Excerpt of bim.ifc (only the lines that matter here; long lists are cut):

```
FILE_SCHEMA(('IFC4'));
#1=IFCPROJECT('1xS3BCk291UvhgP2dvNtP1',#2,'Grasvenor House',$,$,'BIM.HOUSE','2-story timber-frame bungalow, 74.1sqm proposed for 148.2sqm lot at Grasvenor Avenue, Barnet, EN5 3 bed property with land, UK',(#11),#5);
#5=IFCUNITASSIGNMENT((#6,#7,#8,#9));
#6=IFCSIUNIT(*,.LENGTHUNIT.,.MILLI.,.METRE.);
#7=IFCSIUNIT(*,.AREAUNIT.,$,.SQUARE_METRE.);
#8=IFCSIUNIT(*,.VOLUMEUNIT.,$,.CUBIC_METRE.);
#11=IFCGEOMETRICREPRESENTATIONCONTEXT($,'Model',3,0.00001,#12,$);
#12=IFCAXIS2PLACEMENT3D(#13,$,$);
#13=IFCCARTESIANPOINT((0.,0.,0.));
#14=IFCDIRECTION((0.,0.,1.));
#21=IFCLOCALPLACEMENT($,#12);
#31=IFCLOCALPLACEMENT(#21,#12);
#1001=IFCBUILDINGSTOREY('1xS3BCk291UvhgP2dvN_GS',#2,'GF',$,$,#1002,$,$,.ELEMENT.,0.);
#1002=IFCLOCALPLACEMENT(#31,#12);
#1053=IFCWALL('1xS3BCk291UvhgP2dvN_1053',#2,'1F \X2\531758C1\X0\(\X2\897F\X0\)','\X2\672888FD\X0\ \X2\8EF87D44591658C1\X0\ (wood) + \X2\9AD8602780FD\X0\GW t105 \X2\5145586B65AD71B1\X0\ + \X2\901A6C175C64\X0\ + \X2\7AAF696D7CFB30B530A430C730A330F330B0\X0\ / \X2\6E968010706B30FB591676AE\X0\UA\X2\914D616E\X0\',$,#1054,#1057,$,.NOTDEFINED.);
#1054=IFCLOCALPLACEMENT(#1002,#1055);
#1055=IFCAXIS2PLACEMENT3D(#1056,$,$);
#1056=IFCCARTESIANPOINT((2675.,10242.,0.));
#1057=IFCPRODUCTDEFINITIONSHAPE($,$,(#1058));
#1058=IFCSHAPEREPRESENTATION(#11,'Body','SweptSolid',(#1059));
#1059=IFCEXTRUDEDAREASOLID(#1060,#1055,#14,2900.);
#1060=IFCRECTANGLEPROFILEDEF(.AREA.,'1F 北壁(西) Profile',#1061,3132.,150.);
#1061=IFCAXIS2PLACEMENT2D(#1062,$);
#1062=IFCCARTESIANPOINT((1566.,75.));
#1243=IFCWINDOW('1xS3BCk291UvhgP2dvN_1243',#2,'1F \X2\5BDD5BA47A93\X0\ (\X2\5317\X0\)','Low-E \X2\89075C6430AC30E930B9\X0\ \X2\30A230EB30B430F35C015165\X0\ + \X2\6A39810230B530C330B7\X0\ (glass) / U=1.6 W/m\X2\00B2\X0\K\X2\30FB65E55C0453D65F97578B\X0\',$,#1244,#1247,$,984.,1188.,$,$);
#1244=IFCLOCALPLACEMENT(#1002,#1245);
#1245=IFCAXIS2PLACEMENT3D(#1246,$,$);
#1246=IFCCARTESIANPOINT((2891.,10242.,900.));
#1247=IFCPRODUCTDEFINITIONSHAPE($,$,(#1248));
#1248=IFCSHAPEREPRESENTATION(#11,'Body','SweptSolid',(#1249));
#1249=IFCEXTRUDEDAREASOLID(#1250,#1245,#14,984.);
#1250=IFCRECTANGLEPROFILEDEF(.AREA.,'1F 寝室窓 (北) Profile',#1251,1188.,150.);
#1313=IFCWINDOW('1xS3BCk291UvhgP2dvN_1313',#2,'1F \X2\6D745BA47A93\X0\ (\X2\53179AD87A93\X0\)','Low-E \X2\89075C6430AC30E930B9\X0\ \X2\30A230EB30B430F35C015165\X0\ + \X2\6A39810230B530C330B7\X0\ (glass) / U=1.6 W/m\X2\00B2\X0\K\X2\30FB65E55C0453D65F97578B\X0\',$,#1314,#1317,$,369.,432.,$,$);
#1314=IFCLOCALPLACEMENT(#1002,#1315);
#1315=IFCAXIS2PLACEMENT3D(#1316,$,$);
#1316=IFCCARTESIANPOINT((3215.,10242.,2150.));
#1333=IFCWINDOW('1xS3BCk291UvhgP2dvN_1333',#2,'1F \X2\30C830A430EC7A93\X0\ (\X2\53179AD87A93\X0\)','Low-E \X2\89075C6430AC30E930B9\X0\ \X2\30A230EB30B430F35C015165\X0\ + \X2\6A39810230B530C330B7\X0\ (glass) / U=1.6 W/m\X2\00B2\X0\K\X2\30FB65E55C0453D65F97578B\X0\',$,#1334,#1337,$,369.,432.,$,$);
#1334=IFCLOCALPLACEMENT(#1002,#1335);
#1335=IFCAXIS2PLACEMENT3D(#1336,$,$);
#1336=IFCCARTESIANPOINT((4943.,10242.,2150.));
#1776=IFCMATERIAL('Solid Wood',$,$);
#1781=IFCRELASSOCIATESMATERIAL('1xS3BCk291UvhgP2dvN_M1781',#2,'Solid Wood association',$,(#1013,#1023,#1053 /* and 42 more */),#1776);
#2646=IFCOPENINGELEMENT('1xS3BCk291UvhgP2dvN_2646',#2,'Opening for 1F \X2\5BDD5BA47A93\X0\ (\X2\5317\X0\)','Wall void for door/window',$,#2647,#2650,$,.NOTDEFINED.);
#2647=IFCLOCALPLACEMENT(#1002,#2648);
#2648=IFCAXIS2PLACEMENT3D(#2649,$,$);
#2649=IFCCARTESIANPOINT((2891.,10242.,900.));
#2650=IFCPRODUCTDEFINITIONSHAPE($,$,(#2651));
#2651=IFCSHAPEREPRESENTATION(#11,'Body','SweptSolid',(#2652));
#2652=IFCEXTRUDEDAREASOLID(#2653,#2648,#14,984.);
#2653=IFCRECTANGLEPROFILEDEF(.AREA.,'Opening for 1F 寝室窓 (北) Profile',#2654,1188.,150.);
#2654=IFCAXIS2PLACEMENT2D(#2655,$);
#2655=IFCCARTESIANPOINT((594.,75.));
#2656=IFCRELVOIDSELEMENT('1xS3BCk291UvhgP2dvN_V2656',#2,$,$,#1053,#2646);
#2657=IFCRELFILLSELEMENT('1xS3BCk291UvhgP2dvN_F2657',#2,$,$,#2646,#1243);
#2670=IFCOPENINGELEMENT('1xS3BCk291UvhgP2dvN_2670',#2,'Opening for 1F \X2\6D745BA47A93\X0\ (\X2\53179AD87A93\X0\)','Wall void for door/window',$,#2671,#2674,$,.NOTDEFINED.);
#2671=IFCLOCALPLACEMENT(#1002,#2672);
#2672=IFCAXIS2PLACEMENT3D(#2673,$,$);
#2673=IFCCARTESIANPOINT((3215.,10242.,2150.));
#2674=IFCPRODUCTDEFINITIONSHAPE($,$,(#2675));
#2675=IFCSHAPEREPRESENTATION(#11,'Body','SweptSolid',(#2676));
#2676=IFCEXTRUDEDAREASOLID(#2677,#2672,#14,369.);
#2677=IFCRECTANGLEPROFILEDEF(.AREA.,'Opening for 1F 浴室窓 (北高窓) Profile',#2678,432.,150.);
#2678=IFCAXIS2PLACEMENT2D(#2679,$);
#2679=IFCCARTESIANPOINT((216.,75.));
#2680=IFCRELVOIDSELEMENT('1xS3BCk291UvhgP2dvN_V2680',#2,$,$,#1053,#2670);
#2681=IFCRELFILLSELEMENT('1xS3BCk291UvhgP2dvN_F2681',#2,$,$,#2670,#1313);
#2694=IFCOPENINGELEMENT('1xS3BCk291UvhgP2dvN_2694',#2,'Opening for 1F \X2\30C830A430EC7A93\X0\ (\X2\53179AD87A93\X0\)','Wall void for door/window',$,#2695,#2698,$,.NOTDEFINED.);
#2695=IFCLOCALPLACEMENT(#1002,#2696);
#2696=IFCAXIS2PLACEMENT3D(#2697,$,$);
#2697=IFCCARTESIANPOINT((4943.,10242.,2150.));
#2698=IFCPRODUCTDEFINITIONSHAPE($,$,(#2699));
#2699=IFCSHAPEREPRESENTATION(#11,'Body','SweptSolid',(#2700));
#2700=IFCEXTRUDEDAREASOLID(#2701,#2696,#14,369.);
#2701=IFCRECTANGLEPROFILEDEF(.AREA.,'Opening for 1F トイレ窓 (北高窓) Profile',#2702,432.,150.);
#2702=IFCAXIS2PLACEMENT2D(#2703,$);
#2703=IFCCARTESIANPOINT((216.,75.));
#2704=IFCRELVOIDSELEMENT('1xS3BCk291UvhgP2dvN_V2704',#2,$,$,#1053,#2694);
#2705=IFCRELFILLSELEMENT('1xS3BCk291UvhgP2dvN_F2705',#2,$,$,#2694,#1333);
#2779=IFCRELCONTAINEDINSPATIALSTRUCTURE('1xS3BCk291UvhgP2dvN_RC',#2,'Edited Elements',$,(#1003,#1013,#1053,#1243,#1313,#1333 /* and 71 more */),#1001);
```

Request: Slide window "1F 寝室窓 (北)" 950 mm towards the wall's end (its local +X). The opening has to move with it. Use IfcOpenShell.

```python
import ifcopenshell
import ifcopenshell.api.geometry
import ifcopenshell.util.placement

model = ifcopenshell.open("bim.ifc")

window = model.by_guid("1xS3BCk291UvhgP2dvN_1243")
opening = window.FillsVoids[0].RelatingOpeningElement
wall = opening.VoidsElements[0].RelatingBuildingElement

wall_matrix = ifcopenshell.util.placement.get_local_placement(wall.ObjectPlacement)
shift = wall_matrix[:3, 0] * 950.0
before = ifcopenshell.util.placement.get_local_placement(window.ObjectPlacement)[:3, 3].copy()

# The window is not placed relative to its opening, so move both.
for product in (opening, window):
    matrix = ifcopenshell.util.placement.get_local_placement(product.ObjectPlacement)
    matrix[:3, 3] += shift
    ifcopenshell.api.geometry.edit_object_placement(model, product=product, matrix=matrix, is_si=False)

after = ifcopenshell.util.placement.get_local_placement(window.ObjectPlacement)[:3, 3]
print("window moved by", (after - before).round(3) + 0.0)

model.write("bim_edited.ifc")
```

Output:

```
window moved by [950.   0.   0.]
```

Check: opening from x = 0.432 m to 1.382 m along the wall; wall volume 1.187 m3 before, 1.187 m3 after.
